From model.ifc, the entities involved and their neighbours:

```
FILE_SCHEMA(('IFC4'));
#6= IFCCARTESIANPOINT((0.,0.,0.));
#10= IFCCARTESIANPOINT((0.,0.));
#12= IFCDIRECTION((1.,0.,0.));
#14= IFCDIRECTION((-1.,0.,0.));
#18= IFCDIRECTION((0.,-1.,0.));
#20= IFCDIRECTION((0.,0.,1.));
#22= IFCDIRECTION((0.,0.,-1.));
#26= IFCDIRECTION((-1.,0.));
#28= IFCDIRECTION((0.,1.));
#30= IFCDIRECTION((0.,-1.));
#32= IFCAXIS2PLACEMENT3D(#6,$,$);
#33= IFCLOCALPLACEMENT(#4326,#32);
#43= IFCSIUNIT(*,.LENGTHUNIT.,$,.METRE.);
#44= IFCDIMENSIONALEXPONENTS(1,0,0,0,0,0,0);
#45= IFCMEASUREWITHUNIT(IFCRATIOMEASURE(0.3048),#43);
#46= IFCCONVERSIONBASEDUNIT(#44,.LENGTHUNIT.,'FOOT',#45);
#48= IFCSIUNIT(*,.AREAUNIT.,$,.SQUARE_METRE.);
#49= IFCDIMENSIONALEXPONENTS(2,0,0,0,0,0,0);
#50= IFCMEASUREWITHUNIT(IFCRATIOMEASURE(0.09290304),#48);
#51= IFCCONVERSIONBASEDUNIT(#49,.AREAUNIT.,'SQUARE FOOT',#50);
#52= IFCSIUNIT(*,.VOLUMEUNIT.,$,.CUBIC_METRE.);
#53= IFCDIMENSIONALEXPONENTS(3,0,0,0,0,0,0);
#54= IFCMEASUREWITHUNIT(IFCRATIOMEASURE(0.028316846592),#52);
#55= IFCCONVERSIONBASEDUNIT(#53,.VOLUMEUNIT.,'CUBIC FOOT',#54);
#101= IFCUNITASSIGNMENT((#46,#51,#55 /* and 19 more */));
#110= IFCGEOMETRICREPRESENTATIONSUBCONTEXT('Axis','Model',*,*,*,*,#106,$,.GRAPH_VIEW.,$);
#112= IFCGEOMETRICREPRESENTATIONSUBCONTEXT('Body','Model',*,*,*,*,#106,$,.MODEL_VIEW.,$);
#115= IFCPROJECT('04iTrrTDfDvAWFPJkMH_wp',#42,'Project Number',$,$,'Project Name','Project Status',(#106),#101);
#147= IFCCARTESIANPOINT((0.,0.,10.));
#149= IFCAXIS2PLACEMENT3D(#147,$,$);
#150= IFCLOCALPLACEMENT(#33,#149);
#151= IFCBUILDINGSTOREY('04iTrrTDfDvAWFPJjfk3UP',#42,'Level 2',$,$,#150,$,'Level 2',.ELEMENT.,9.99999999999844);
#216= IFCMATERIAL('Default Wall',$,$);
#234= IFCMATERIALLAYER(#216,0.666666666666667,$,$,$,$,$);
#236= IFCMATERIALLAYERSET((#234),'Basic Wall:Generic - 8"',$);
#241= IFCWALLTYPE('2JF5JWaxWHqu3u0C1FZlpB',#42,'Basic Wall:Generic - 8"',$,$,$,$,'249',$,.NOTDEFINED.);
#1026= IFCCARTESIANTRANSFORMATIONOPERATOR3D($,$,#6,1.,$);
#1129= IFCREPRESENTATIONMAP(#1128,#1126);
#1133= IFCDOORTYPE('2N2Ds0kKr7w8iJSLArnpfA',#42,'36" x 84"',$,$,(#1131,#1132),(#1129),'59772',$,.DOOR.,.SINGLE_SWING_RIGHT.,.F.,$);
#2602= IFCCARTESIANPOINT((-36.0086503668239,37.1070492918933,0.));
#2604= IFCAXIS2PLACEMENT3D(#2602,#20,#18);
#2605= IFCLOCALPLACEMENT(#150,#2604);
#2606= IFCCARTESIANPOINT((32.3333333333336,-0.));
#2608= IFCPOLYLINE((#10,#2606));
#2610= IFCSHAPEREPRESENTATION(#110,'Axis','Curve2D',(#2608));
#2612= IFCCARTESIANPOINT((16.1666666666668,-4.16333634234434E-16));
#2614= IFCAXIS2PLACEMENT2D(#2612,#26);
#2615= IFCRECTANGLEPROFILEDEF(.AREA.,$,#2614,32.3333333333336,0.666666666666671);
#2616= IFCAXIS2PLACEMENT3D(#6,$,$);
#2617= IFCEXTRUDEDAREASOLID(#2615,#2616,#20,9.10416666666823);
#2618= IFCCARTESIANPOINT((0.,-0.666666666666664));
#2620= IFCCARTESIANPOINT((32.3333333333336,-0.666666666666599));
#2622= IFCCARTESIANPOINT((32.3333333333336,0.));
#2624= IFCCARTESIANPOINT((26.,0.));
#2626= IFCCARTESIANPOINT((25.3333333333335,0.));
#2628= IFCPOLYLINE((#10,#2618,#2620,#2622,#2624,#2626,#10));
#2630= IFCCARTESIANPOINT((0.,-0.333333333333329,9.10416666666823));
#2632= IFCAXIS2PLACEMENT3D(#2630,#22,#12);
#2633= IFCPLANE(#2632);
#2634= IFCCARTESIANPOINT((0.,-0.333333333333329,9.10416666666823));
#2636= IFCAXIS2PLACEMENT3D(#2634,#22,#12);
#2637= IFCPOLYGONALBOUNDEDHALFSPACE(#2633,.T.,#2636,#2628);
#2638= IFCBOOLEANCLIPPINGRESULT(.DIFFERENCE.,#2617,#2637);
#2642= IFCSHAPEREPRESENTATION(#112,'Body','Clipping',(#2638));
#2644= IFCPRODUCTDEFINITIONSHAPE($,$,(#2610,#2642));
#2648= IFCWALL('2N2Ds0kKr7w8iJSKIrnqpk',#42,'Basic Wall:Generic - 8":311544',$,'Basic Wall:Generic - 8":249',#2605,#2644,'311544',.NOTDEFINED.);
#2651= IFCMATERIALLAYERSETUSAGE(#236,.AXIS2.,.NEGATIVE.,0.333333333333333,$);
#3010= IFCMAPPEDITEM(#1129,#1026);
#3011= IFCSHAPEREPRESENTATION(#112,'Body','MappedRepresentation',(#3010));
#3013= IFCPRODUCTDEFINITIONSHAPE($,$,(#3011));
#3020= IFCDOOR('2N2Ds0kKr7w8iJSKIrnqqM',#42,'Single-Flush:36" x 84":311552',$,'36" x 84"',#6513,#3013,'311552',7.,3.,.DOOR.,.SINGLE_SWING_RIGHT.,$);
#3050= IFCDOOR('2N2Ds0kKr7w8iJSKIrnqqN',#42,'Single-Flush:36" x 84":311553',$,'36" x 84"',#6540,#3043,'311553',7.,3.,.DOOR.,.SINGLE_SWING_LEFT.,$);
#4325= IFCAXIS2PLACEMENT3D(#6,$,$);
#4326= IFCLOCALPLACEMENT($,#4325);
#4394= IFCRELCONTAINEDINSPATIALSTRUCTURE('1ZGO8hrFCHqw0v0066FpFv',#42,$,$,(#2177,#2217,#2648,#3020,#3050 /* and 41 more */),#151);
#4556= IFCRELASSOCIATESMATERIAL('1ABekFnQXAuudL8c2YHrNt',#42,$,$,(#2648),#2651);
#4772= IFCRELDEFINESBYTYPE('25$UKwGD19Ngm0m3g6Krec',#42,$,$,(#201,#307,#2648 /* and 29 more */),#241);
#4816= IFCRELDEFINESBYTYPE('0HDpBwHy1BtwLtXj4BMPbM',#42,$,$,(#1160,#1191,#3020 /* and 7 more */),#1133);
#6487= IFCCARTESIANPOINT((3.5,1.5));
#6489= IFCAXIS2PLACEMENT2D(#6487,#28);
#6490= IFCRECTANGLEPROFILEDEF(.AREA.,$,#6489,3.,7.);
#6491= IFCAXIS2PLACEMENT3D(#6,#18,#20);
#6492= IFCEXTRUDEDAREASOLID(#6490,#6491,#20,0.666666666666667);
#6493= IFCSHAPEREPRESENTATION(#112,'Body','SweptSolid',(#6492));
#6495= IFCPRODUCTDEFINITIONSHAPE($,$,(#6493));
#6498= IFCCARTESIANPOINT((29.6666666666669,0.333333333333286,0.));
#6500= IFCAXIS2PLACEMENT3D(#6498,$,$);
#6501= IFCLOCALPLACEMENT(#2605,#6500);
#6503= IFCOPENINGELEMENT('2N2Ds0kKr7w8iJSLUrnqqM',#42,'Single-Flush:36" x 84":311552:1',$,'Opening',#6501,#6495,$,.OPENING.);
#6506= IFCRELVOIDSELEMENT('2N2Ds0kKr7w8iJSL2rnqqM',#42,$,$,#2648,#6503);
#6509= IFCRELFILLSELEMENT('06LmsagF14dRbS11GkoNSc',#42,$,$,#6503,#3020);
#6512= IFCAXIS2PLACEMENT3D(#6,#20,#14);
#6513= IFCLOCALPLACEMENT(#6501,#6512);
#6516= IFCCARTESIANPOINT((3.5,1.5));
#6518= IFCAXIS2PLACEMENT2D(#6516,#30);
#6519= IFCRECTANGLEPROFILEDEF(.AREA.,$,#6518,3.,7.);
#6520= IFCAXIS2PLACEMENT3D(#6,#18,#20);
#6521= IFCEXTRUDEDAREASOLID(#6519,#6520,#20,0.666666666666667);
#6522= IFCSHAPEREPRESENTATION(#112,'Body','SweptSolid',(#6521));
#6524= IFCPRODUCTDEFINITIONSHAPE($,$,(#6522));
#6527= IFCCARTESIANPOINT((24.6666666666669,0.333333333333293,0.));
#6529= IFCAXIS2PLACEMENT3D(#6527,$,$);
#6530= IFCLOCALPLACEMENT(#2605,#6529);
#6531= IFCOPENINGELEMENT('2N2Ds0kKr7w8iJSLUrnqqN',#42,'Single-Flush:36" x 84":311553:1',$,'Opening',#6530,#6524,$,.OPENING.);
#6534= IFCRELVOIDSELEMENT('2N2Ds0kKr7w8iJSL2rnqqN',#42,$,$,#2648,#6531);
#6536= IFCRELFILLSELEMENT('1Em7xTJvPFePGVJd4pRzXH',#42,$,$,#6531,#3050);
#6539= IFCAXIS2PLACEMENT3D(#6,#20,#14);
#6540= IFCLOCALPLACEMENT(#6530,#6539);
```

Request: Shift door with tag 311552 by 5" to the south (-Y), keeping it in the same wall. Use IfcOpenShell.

```python
import ifcopenshell
import ifcopenshell.api.geometry
import ifcopenshell.util.placement
import ifcopenshell.util.unit

model = ifcopenshell.open("model.ifc")
unit_scale = ifcopenshell.util.unit.calculate_unit_scale(model)

door = model.by_guid("2N2Ds0kKr7w8iJSKIrnqqM")
opening = door.FillsVoids[0].RelatingOpeningElement
wall = opening.VoidsElements[0].RelatingBuildingElement

wall_matrix = ifcopenshell.util.placement.get_local_placement(wall.ObjectPlacement)
shift = wall_matrix[:3, 0] * 5 * 0.0254 / unit_scale
before = ifcopenshell.util.placement.get_local_placement(door.ObjectPlacement)[:3, 3].copy()

# The door is placed relative to its opening, so it follows when the opening moves.
matrix = ifcopenshell.util.placement.get_local_placement(opening.ObjectPlacement)
matrix[:3, 3] += shift
ifcopenshell.api.geometry.edit_object_placement(
    model, product=opening, matrix=matrix, is_si=False, should_transform_children=True
)

after = ifcopenshell.util.placement.get_local_placement(door.ObjectPlacement)[:3, 3]
print("door moved by", (after - before).round(3) + 0.0)

model.write("model_v2.ifc")
```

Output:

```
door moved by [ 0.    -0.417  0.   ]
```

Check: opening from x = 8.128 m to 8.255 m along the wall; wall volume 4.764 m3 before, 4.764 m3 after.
